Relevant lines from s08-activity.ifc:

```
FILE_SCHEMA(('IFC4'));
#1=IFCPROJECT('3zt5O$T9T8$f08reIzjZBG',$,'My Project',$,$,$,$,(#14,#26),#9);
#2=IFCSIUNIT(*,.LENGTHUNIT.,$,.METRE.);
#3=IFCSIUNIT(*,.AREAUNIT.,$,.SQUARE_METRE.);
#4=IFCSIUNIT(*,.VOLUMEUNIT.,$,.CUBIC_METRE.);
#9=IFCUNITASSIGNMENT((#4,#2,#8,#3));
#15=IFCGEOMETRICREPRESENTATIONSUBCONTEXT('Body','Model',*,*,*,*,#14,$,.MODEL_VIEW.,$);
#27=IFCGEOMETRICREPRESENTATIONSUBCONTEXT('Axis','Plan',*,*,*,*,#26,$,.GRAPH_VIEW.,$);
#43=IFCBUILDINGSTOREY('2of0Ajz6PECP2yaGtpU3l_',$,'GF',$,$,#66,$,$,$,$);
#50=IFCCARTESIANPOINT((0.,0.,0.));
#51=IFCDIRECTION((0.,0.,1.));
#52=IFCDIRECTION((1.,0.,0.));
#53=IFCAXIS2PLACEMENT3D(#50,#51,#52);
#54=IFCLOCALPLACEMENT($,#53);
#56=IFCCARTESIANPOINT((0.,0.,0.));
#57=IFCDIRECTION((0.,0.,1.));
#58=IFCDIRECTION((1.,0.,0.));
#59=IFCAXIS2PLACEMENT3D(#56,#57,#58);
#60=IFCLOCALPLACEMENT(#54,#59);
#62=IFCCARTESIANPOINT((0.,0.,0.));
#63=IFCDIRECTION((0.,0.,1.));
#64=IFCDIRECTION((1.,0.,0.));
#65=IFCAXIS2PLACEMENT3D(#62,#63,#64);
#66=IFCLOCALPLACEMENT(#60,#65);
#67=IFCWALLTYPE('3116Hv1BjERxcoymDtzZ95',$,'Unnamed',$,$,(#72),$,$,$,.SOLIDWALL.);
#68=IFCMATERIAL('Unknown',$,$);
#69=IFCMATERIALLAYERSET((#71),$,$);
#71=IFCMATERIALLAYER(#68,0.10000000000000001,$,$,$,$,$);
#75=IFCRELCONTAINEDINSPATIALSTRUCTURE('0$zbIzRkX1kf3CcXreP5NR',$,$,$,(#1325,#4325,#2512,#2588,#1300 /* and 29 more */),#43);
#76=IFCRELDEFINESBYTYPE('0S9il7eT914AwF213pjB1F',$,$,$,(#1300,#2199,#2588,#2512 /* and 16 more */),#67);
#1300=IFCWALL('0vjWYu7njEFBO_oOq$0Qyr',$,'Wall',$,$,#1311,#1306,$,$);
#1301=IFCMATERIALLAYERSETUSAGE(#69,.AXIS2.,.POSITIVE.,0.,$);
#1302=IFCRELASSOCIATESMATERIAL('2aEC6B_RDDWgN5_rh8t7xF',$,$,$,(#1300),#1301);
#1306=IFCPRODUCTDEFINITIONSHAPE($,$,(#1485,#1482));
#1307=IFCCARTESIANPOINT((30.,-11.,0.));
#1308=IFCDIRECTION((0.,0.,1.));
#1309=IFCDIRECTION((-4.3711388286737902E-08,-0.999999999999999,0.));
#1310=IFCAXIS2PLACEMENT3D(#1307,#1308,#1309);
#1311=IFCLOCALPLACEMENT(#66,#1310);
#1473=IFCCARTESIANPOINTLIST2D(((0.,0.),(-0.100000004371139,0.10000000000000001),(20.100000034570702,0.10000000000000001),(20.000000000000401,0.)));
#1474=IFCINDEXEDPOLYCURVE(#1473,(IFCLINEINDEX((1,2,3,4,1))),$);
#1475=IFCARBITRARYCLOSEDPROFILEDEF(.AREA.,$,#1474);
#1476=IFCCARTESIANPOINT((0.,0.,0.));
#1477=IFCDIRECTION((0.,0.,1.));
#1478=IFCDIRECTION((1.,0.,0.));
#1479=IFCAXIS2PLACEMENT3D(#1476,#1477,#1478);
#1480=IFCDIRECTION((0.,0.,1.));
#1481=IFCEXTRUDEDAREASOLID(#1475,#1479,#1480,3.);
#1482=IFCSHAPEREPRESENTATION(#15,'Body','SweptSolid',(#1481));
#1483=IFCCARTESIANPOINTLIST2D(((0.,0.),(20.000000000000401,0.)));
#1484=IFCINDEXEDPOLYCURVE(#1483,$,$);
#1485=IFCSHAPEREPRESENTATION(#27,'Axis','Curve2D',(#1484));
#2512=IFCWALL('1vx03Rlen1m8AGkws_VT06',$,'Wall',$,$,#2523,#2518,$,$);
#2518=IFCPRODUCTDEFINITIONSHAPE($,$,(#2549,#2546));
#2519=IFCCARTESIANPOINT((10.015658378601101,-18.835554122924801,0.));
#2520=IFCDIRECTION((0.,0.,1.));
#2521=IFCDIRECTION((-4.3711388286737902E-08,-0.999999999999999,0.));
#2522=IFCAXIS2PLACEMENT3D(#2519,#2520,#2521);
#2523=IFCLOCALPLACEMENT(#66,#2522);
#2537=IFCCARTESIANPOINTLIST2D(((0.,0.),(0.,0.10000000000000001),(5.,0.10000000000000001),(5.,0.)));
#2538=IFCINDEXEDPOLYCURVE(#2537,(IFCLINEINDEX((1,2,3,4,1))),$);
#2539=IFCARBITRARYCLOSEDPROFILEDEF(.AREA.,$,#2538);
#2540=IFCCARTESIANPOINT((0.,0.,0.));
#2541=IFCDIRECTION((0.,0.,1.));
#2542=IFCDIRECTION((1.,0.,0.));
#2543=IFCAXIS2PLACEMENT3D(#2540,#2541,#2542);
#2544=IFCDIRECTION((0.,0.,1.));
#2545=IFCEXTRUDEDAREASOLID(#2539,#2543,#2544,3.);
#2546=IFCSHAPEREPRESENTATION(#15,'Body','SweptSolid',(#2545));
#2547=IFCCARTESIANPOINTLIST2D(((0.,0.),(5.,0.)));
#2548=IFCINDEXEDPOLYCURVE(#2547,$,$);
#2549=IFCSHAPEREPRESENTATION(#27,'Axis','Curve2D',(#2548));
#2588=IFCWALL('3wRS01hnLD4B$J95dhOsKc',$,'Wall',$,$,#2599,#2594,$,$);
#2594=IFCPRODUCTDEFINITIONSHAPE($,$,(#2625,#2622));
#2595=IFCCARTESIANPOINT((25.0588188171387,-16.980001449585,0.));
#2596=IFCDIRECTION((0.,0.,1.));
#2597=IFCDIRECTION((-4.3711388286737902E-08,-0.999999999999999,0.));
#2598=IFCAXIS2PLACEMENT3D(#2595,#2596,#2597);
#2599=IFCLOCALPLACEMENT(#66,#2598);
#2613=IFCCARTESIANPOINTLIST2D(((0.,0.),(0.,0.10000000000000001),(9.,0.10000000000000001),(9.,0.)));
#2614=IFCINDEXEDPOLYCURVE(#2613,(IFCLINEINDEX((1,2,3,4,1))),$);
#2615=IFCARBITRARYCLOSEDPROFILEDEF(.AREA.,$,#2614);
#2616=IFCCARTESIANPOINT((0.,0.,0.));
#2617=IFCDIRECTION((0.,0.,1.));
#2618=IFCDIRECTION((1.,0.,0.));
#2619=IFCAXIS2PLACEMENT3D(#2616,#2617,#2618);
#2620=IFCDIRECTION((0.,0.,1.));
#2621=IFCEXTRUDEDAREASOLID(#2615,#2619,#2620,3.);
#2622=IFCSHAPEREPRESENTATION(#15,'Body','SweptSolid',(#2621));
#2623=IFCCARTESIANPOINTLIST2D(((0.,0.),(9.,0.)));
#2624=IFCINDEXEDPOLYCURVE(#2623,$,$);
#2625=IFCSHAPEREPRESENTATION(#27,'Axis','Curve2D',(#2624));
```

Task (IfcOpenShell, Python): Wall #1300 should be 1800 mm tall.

```python
import ifcopenshell
import ifcopenshell.geom
import ifcopenshell.util.representation
import ifcopenshell.util.shape
import ifcopenshell.util.unit

model = ifcopenshell.open("s08-activity.ifc")
unit_scale = ifcopenshell.util.unit.calculate_unit_scale(model)
settings = ifcopenshell.geom.settings()


def volume(element):
    """Net volume in cubic metres, openings subtracted."""
    shape = ifcopenshell.geom.create_shape(settings, element)
    return ifcopenshell.util.shape.get_volume(shape.geometry)


wall = model.by_id(1300)
before = volume(wall)

body = ifcopenshell.util.representation.get_representation(wall, "Model", "Body")
solid = body.Items[0]
old_height = solid.Depth
solid.Depth = 1.8 / unit_scale
after = volume(wall)

print(f"height {old_height:g} -> {solid.Depth:g}, volume {before:.3f} -> {after:.3f} m3")

model.write("s08-activity_rev.ifc")
```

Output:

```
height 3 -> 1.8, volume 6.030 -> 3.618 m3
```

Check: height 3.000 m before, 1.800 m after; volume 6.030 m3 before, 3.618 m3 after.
